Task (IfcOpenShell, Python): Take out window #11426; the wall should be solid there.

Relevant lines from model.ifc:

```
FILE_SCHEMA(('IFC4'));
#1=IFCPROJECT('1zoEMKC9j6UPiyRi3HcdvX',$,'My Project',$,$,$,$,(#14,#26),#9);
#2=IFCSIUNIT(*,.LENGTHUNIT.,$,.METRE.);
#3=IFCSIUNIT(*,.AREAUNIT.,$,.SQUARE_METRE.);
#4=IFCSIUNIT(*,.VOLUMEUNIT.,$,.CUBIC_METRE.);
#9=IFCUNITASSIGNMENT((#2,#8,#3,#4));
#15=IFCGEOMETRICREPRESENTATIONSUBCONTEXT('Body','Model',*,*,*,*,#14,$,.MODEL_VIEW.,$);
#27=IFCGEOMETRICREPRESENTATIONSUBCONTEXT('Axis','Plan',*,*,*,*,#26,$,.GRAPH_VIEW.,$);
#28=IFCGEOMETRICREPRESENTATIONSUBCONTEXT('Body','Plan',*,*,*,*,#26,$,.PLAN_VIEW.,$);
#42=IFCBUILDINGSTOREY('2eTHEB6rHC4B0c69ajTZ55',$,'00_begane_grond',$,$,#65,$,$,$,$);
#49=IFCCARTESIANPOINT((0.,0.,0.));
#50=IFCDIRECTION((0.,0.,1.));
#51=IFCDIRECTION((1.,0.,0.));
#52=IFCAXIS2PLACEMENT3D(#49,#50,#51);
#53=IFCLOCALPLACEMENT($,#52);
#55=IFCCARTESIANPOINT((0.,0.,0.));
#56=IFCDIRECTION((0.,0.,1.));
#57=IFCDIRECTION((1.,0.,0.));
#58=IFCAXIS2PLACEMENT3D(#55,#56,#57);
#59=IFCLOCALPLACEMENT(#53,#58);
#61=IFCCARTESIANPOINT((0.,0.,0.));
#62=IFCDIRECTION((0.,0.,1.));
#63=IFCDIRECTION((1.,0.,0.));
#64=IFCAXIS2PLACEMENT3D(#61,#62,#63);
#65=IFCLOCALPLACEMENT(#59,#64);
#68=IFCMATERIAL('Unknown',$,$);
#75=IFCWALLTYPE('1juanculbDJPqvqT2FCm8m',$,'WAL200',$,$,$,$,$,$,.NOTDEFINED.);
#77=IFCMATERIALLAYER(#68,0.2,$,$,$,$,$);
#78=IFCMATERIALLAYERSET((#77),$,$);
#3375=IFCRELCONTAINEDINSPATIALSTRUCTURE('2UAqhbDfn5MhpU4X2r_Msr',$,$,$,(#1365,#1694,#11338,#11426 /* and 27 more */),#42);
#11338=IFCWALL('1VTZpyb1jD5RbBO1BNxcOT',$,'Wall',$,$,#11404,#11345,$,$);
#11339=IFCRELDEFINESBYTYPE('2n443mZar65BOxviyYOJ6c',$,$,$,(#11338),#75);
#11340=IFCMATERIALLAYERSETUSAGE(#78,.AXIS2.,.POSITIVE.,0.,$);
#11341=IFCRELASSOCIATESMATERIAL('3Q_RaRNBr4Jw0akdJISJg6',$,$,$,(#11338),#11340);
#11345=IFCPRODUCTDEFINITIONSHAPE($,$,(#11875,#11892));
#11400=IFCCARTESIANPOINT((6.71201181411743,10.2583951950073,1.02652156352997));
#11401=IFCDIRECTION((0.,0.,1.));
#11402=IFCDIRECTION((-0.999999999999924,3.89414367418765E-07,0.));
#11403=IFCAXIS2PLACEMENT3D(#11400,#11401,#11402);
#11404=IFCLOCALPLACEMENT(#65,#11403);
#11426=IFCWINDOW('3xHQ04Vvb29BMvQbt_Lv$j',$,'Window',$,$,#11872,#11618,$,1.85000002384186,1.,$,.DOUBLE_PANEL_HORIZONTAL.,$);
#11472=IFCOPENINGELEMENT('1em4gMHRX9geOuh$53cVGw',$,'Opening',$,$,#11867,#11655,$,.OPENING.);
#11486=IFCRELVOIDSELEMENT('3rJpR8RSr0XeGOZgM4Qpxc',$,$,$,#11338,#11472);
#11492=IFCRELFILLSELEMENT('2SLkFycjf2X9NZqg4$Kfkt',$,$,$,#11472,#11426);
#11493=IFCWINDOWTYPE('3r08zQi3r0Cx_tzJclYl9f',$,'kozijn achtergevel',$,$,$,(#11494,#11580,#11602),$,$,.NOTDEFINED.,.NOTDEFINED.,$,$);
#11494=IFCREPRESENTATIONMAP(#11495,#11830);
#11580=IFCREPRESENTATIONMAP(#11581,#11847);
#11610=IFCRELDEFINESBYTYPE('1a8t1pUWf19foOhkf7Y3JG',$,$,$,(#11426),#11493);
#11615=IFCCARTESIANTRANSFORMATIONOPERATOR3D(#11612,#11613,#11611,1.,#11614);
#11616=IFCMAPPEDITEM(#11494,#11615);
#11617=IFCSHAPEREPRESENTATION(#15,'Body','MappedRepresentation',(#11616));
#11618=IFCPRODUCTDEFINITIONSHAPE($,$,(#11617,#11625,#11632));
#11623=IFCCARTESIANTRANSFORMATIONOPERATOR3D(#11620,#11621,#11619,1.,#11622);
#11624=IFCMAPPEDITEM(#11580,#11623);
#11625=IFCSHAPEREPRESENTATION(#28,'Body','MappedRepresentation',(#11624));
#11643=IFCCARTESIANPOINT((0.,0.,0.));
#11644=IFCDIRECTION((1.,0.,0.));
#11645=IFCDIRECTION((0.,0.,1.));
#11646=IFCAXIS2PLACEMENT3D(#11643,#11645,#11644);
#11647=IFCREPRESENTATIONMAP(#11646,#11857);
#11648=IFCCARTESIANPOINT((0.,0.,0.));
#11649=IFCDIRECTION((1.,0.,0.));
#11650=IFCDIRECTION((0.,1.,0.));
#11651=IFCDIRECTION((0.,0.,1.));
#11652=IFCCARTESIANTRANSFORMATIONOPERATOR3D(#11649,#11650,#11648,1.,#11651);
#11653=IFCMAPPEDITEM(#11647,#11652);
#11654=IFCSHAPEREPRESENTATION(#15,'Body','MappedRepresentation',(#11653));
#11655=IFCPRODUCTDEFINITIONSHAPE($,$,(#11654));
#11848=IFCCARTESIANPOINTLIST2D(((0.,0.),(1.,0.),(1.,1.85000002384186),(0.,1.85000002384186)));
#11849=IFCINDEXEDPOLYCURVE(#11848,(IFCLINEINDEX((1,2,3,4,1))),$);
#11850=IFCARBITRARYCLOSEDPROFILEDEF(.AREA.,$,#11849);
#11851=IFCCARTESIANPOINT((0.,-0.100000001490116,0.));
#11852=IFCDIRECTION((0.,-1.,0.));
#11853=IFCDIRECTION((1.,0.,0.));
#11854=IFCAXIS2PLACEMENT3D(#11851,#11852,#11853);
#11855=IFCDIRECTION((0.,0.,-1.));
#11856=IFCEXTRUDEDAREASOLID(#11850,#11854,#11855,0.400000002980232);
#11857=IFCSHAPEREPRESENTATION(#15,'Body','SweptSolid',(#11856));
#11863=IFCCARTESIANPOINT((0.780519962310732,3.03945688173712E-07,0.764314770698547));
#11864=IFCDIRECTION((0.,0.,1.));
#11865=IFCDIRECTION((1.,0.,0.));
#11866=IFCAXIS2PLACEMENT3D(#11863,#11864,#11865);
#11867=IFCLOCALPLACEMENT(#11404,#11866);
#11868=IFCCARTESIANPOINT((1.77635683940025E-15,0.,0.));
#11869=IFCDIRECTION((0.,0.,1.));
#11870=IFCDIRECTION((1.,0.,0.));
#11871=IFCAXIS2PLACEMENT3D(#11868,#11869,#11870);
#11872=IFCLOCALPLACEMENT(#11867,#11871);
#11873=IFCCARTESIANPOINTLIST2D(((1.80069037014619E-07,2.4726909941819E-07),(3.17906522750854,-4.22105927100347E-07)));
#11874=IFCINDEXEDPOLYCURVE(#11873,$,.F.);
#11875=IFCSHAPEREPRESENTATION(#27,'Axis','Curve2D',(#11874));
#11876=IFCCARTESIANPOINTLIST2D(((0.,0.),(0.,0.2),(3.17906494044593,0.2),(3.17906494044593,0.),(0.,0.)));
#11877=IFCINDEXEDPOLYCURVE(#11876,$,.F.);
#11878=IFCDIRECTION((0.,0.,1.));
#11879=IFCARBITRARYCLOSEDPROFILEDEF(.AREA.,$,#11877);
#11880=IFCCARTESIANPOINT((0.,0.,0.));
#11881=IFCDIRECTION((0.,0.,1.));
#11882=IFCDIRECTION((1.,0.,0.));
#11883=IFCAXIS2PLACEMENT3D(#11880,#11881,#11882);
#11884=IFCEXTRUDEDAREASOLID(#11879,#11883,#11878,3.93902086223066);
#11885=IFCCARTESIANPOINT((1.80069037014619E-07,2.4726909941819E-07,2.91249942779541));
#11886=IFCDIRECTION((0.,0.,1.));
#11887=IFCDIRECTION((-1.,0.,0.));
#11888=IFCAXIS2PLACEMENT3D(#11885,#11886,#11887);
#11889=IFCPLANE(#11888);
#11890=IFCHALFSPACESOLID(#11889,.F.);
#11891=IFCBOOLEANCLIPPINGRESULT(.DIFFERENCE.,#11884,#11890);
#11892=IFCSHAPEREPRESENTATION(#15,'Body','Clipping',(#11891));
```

```python
import ifcopenshell
import ifcopenshell.api.feature
import ifcopenshell.api.root
import ifcopenshell.geom
import ifcopenshell.util.shape

model = ifcopenshell.open("model.ifc")
settings = ifcopenshell.geom.settings()


def volume(element):
    """Net volume in cubic metres, openings subtracted."""
    shape = ifcopenshell.geom.create_shape(settings, element)
    return ifcopenshell.util.shape.get_volume(shape.geometry)


window = model.by_id(11426)
opening = window.FillsVoids[0].RelatingOpeningElement
wall = opening.VoidsElements[0].RelatingBuildingElement
before = volume(wall)

ifcopenshell.api.root.remove_product(model, product=window)
ifcopenshell.api.feature.remove_feature(model, feature=opening)

after = volume(wall)

print(f"wall volume {before:.3f} -> {after:.3f} m3")

model.write("model_v2.ifc")
```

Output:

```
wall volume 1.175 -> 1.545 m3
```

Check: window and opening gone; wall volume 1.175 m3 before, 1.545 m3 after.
